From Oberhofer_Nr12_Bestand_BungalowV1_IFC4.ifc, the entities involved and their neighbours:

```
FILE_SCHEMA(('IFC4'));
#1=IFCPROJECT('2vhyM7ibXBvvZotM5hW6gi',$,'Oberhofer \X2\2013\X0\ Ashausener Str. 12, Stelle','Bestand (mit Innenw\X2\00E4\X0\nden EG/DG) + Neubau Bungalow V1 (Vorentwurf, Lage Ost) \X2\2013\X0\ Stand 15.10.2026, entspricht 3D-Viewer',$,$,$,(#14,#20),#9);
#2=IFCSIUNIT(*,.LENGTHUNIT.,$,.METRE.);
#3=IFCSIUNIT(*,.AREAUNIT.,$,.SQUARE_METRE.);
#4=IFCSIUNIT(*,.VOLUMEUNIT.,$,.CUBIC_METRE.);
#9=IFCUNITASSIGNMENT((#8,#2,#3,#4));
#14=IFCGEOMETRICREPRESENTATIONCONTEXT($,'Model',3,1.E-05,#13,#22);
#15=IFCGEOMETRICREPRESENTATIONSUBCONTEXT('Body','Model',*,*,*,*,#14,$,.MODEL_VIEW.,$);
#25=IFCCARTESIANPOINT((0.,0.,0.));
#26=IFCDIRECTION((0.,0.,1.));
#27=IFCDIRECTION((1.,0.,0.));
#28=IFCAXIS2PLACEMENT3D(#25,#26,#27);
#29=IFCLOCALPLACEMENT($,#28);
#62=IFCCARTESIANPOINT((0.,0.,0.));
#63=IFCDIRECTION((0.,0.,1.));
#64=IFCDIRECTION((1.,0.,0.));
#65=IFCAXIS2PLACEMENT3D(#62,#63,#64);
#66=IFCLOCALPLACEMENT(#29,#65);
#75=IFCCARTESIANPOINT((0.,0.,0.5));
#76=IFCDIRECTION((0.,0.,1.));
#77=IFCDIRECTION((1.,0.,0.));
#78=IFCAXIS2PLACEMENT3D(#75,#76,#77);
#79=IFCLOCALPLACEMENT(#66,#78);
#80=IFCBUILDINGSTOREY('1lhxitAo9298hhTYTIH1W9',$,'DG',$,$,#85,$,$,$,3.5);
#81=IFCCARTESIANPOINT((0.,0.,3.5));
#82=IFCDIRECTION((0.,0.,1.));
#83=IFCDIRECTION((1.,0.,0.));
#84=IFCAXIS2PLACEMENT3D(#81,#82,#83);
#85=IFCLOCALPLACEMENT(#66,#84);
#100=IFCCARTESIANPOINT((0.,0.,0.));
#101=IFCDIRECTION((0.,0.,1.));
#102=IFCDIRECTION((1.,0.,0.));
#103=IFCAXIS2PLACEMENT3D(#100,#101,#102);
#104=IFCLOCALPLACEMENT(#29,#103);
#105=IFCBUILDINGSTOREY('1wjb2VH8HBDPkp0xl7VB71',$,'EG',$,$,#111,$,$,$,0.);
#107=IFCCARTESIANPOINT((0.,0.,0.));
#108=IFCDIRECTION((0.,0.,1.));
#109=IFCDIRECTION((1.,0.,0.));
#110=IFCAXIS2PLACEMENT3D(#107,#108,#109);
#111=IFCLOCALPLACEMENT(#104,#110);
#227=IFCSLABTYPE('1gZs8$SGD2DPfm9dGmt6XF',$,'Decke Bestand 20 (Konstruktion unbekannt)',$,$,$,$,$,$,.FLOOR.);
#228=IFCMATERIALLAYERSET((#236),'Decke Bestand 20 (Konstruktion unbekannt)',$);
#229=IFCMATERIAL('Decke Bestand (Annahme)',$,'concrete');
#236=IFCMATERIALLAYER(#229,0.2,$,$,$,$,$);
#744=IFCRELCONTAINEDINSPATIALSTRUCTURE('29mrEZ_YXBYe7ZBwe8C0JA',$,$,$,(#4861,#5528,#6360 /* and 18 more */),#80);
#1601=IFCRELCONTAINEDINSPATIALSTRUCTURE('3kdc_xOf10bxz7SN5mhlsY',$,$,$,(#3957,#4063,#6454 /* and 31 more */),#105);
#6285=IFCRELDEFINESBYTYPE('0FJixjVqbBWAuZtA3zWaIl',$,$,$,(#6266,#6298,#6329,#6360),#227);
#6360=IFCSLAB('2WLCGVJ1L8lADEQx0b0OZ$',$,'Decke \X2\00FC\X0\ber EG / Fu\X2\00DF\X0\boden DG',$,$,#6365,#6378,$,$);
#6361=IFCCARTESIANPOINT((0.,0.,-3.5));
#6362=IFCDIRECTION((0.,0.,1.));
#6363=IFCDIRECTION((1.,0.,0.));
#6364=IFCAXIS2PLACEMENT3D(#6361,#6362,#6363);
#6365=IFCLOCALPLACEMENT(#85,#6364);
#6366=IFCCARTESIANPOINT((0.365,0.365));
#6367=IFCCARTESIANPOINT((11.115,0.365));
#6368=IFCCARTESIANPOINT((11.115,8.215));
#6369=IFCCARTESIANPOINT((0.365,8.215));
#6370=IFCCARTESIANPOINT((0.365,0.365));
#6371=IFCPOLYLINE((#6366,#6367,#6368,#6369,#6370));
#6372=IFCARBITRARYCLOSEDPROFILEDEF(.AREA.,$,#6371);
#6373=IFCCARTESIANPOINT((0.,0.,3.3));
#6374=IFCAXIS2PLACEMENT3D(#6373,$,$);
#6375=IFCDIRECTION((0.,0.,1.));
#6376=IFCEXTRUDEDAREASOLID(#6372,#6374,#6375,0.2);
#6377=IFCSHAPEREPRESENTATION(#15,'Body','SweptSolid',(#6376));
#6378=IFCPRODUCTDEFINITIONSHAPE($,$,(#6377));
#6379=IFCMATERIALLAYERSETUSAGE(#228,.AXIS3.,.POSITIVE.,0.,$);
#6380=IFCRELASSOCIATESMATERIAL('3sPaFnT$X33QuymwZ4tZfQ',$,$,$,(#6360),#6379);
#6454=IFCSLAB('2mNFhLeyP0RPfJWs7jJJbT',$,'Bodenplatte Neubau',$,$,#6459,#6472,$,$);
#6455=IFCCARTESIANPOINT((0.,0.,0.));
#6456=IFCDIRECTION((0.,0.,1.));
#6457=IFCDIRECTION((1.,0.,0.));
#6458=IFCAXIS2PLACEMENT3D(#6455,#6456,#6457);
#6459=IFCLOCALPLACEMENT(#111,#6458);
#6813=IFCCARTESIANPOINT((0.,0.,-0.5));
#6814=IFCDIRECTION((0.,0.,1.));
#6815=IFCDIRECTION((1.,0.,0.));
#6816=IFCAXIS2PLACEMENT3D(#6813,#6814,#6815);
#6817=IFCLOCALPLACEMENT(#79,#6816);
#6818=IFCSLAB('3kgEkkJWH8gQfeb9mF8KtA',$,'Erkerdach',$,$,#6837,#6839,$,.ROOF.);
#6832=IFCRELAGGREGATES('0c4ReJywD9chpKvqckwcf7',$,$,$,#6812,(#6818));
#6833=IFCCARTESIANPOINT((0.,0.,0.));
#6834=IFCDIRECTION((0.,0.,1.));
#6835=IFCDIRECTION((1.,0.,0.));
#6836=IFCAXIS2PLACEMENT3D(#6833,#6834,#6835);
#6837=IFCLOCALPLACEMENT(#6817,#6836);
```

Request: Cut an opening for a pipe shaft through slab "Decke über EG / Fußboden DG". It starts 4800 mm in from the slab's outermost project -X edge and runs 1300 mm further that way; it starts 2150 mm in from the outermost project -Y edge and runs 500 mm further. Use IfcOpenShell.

```python
import numpy as np
import ifcopenshell
import ifcopenshell.api.feature
import ifcopenshell.api.geometry
import ifcopenshell.api.root
import ifcopenshell.geom
import ifcopenshell.util.placement
import ifcopenshell.util.representation
import ifcopenshell.util.shape
import ifcopenshell.util.unit

model = ifcopenshell.open("Oberhofer_Nr12_Bestand_BungalowV1_IFC4.ifc")
unit_scale = ifcopenshell.util.unit.calculate_unit_scale(model)
settings = ifcopenshell.geom.settings()


def volume(element):
    """Net volume in cubic metres, openings subtracted."""
    shape = ifcopenshell.geom.create_shape(settings, element)
    return ifcopenshell.util.shape.get_volume(shape.geometry)


slab = model.by_guid("2WLCGVJ1L8lADEQx0b0OZ$")
before = volume(slab)

# Extent in the slab's own axes, in metres. The edges named are its -X and -Y sides.
slab_shape = ifcopenshell.geom.create_shape(settings, slab)
vertices = ifcopenshell.util.shape.get_vertices(slab_shape.geometry)
x_min, y_min, bottom = vertices.min(axis=0)
top = vertices[:, 2].max()

opening = ifcopenshell.api.root.create_entity(model, ifc_class="IfcOpeningElement", name="Pipe shaft opening", predefined_type="OPENING")
context = ifcopenshell.util.representation.get_context(model, "Model", "Body", "MODEL_VIEW")
width, depth = 1.3, 0.5
outline = [(0.0, 0.0), (width, 0.0), (width, depth), (0.0, depth), (0.0, 0.0)]
# Overshoot both faces by 50 mm so the cut is clean.
shape = ifcopenshell.api.geometry.add_slab_representation(
    model, context=context, depth=top - bottom + 0.1, polyline=outline
)
ifcopenshell.api.geometry.assign_representation(model, product=opening, representation=shape)

matrix = ifcopenshell.util.placement.get_local_placement(slab.ObjectPlacement)
matrix[:, 3] = matrix @ np.append(np.array([x_min + 4.8, y_min + 2.15, bottom - 0.05]) / unit_scale, 1.0)
ifcopenshell.api.geometry.edit_object_placement(model, product=opening, matrix=matrix, is_si=False)
ifcopenshell.api.feature.add_feature(model, feature=opening, element=slab)

after = volume(slab)

print(f"slab volume {before:.3f} -> {after:.3f} m3")

model.write("Oberhofer_Nr12_Bestand_BungalowV1_IFC4_v2.ifc")
```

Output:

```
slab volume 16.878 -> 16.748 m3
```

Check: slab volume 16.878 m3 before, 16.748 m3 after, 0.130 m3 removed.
